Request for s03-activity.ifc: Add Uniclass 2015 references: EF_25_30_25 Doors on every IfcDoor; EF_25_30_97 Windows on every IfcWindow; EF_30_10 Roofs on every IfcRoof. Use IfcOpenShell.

First a look at what the model holds.

```python
import ifcopenshell

model = ifcopenshell.open("s03-activity.ifc")
print(model.schema)
print("classifications:", [c.Name for c in model.by_type("IfcClassification")])
for ifc_class in ("IfcDoor", "IfcRoof", "IfcStair", "IfcWall", "IfcWindow"):
    print(ifc_class, len(model.by_type(ifc_class)))
```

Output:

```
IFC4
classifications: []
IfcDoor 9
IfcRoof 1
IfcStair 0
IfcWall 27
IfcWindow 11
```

```python
import ifcopenshell
import ifcopenshell.api.classification

model = ifcopenshell.open("s03-activity.ifc")

system = ifcopenshell.api.classification.add_classification(model, classification="Uniclass 2015")

codes = {
    "IfcDoor": ("EF_25_30_25", "Doors"),
    "IfcWindow": ("EF_25_30_97", "Windows"),
    "IfcRoof": ("EF_30_10", "Roofs"),
}
for ifc_class, (code, name) in codes.items():
    products = model.by_type(ifc_class)
    ifcopenshell.api.classification.add_reference(
        model, products=products, classification=system, identification=code, name=name
    )
    print(code, len(products))

model.write("s03-activity_updated.ifc")
```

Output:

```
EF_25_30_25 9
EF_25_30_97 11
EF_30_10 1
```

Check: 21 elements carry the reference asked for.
